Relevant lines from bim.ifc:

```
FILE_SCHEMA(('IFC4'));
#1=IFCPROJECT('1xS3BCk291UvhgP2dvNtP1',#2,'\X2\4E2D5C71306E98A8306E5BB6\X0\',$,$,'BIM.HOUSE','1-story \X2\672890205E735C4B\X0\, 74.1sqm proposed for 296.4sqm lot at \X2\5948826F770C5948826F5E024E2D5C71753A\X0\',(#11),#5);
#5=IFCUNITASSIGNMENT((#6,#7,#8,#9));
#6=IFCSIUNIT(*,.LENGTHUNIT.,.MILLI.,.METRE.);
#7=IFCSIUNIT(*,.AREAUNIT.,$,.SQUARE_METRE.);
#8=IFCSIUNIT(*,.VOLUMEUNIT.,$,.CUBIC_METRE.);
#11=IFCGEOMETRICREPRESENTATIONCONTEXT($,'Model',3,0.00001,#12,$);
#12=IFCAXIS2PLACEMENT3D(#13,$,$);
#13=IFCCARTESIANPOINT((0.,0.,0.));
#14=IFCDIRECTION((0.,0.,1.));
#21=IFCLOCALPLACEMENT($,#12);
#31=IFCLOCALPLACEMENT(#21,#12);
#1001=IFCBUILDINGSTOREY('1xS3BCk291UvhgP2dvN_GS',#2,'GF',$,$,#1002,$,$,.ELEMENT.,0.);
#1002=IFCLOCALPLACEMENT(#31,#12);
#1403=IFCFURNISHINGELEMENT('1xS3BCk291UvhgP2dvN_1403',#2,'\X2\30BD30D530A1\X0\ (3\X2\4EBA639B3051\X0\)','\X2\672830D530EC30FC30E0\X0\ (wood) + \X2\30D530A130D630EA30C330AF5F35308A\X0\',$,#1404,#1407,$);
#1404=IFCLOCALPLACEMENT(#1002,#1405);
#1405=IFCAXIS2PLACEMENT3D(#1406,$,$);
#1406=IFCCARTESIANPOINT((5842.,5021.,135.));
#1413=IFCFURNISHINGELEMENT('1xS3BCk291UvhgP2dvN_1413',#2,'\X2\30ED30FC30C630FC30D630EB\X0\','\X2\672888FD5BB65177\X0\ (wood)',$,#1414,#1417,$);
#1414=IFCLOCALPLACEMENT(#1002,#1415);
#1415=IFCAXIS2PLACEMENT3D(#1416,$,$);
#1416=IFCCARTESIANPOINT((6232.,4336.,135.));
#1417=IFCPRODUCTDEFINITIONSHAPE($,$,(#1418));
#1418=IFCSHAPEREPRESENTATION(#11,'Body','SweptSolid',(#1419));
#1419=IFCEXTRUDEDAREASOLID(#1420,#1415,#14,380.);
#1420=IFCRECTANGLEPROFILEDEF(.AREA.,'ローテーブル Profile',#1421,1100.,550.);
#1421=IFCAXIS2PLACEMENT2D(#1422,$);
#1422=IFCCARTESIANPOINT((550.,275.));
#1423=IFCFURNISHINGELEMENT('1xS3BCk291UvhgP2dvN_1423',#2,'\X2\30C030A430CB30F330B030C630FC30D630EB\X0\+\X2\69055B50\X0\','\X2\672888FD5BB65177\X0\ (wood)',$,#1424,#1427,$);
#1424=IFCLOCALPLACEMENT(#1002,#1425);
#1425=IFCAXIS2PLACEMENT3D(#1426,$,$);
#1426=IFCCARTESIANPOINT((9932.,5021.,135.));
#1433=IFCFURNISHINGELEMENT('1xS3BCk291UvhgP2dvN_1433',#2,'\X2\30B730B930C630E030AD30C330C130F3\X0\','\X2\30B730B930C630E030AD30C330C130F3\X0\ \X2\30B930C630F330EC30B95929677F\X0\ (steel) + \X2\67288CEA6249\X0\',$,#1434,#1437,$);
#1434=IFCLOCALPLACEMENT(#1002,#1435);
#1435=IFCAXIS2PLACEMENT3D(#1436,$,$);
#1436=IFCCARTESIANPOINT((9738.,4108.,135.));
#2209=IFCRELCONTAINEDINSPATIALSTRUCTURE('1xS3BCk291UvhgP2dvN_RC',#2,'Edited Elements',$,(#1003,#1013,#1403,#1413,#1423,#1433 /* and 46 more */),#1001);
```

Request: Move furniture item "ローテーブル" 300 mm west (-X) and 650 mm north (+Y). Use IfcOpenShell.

```python
import ifcopenshell
import ifcopenshell.api.geometry
import ifcopenshell.util.placement
import ifcopenshell.util.unit

model = ifcopenshell.open("bim.ifc")
unit_scale = ifcopenshell.util.unit.calculate_unit_scale(model)

item = model.by_guid("1xS3BCk291UvhgP2dvN_1413")
matrix = ifcopenshell.util.placement.get_local_placement(item.ObjectPlacement)
matrix[0, 3] -= 0.3 / unit_scale
matrix[1, 3] += 0.65 / unit_scale
ifcopenshell.api.geometry.edit_object_placement(model, product=item, matrix=matrix, is_si=False)

print(ifcopenshell.util.placement.get_local_placement(item.ObjectPlacement).round(3) + 0.0)

model.write("bim_updated.ifc")
```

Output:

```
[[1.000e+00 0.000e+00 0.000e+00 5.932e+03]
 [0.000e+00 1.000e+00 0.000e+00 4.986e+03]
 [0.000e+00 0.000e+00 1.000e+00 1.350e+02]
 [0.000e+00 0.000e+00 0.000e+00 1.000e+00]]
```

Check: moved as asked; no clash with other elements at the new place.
